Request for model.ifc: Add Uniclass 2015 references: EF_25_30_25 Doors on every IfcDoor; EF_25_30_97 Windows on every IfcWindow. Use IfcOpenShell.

First a look at what the model holds.

```python
import ifcopenshell

model = ifcopenshell.open("model.ifc")
print(model.schema)
print("classifications:", [c.Name for c in model.by_type("IfcClassification")])
for ifc_class in ("IfcDoor", "IfcRoof", "IfcStair", "IfcWall", "IfcWindow"):
    print(ifc_class, len(model.by_type(ifc_class)))
```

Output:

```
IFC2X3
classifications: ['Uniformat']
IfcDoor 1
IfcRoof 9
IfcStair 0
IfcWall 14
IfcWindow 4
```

```python
import ifcopenshell
import ifcopenshell.api.classification

model = ifcopenshell.open("model.ifc")

# IFC2X3 requires Source and Edition and has no link from the project to the system.
system = model.create_entity("IfcClassification", Source="NBS", Edition="2015", Name="Uniclass 2015")

codes = {
    "IfcDoor": ("EF_25_30_25", "Doors"),
    "IfcWindow": ("EF_25_30_97", "Windows"),
}
for ifc_class, (code, name) in codes.items():
    products = model.by_type(ifc_class)
    ifcopenshell.api.classification.add_reference(
        model, products=products, classification=system, identification=code, name=name
    )
    print(code, len(products))

model.write("model_updated.ifc")
```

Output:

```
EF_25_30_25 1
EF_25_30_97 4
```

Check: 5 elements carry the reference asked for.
